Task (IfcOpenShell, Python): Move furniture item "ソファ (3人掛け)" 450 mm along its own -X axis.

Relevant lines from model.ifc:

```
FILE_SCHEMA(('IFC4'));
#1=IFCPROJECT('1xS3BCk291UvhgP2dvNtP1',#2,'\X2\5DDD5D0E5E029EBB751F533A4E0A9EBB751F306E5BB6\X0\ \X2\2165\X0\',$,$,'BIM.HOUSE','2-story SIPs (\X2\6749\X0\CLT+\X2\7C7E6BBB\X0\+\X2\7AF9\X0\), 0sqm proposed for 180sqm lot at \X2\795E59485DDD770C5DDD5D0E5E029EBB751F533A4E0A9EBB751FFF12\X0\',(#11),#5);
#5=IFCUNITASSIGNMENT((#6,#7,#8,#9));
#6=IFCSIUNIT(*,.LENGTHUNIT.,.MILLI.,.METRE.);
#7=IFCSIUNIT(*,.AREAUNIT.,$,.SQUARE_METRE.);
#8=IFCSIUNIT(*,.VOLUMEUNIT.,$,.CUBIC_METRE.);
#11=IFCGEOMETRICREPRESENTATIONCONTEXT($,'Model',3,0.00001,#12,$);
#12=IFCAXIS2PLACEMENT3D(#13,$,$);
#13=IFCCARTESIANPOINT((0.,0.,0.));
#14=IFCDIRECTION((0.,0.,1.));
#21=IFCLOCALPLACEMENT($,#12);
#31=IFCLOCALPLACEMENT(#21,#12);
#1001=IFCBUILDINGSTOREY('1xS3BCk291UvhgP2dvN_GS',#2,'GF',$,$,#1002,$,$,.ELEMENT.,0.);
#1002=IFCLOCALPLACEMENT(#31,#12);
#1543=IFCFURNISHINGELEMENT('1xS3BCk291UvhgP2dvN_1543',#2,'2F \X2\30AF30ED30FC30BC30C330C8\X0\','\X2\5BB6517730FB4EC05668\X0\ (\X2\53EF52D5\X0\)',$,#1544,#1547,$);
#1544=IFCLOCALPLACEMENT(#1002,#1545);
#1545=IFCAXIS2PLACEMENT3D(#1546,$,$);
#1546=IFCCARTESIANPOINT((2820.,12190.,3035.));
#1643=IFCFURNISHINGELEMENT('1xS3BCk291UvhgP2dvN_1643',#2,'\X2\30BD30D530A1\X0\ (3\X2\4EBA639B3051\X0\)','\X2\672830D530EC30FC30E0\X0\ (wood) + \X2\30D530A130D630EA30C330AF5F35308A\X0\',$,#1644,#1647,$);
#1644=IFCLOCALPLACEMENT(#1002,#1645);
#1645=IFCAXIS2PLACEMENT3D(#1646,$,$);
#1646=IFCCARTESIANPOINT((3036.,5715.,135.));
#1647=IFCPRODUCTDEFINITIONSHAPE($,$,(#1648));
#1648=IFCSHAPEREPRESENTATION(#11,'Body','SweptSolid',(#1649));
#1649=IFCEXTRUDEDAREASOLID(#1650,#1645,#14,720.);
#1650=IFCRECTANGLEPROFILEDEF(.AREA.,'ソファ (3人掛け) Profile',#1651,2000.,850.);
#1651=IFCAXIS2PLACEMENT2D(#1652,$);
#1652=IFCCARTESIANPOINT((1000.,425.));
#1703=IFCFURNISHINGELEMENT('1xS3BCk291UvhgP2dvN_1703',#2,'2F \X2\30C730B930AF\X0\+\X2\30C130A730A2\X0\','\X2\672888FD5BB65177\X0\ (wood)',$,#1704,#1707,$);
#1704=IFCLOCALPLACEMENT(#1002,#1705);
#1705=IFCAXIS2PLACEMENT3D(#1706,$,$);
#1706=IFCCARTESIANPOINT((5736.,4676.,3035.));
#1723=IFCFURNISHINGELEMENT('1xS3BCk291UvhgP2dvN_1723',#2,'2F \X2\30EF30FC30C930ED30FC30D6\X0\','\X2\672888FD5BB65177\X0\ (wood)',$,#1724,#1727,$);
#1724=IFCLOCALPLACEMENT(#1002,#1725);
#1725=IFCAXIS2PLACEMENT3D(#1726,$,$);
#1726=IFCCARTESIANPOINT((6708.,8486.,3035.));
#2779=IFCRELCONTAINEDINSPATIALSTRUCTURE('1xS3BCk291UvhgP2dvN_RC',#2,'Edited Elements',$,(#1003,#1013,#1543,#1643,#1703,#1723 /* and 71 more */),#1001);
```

```python
import ifcopenshell
import ifcopenshell.api.geometry
import ifcopenshell.util.placement
import ifcopenshell.util.unit

model = ifcopenshell.open("model.ifc")
unit_scale = ifcopenshell.util.unit.calculate_unit_scale(model)

item = model.by_id(1643)
matrix = ifcopenshell.util.placement.get_local_placement(item.ObjectPlacement)
matrix[:3, 3] -= matrix[:3, 0] * 0.45 / unit_scale
ifcopenshell.api.geometry.edit_object_placement(model, product=item, matrix=matrix, is_si=False)

print(ifcopenshell.util.placement.get_local_placement(item.ObjectPlacement).round(3) + 0.0)

model.write("model_updated.ifc")
```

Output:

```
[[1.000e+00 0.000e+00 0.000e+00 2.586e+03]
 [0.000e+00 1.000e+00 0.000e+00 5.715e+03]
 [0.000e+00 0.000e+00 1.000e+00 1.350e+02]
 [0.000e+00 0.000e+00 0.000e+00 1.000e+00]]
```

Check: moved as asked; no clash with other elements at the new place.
